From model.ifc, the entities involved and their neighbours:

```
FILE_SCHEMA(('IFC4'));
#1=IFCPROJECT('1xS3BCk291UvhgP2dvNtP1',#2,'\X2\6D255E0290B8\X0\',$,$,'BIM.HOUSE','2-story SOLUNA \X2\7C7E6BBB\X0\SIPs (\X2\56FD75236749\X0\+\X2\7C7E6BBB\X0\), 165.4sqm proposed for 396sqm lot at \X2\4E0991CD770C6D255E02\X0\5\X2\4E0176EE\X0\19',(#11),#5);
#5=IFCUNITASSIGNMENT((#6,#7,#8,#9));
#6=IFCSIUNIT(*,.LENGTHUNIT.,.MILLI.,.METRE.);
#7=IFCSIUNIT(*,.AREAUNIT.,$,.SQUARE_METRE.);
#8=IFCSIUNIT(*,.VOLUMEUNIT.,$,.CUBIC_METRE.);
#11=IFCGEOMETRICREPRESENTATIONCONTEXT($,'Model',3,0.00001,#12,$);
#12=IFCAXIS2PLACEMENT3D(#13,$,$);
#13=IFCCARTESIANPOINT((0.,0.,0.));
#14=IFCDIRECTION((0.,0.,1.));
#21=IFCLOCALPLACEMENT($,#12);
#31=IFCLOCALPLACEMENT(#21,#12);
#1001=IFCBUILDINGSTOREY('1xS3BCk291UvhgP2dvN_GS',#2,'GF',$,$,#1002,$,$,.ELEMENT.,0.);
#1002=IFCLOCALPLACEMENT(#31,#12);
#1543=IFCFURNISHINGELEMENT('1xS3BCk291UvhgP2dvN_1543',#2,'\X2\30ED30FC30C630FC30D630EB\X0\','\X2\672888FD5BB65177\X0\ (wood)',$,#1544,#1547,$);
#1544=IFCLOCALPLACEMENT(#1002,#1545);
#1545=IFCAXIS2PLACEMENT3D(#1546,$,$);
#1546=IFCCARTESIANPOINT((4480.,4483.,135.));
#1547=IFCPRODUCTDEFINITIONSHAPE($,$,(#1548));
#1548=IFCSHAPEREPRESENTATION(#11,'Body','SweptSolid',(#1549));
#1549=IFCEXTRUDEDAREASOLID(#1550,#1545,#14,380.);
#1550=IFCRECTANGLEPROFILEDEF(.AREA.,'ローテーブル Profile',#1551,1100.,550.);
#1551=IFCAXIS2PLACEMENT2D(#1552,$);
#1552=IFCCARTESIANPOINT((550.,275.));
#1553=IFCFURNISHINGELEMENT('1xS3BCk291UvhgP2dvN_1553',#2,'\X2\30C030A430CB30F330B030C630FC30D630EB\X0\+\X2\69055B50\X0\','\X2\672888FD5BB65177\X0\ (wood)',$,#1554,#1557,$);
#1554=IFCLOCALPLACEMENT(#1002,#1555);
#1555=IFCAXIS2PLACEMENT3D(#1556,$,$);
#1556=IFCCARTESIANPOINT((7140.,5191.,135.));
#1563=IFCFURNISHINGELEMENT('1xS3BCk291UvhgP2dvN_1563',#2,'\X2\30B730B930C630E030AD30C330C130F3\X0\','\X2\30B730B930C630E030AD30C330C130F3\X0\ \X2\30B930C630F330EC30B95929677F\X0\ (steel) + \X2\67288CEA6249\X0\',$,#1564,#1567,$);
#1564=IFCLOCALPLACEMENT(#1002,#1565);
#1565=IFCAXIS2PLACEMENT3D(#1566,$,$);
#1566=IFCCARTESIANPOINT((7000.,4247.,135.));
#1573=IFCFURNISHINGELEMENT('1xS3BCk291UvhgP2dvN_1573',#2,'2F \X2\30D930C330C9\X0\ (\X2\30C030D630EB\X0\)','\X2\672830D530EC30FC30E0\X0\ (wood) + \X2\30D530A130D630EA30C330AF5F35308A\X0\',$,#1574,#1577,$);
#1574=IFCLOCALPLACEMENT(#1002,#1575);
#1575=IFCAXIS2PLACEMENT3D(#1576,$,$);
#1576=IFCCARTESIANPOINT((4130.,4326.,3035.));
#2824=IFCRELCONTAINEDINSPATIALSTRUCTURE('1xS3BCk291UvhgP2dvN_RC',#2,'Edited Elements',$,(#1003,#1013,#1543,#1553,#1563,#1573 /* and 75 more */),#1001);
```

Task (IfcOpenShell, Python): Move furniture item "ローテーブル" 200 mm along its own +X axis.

```python
import ifcopenshell
import ifcopenshell.api.geometry
import ifcopenshell.util.placement
import ifcopenshell.util.unit

model = ifcopenshell.open("model.ifc")
unit_scale = ifcopenshell.util.unit.calculate_unit_scale(model)

item = model.by_id(1543)
matrix = ifcopenshell.util.placement.get_local_placement(item.ObjectPlacement)
matrix[:3, 3] += matrix[:3, 0] * 0.2 / unit_scale
ifcopenshell.api.geometry.edit_object_placement(model, product=item, matrix=matrix, is_si=False)

print(ifcopenshell.util.placement.get_local_placement(item.ObjectPlacement).round(3) + 0.0)

model.write("model-out.ifc")
```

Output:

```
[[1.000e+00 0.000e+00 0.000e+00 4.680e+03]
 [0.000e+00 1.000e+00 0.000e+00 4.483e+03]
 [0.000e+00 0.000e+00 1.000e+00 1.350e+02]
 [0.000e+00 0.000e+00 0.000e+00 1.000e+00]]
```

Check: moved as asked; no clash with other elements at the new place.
